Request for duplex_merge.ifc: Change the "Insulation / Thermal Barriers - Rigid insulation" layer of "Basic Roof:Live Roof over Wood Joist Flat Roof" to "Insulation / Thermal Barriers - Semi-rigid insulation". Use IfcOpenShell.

First a look at what the model holds.

```python
import ifcopenshell
import ifcopenshell.util.element

model = ifcopenshell.open("duplex_merge.ifc")
print(model.schema)
for layer_set in model.by_type("IfcMaterialLayerSet"):
    if layer_set.LayerSetName == "Basic Roof:Live Roof over Wood Joist Flat Roof":
        for layer in layer_set.MaterialLayers:
            print(layer.id(), layer.Material and layer.Material.Name, layer.LayerThickness, sep=" | ")
        print(len(ifcopenshell.util.element.get_elements_by_material(model, layer_set)), "elements and types use it")
print(sorted(m.Name for m in model.by_type("IfcMaterial") if m.Name)[:60])
```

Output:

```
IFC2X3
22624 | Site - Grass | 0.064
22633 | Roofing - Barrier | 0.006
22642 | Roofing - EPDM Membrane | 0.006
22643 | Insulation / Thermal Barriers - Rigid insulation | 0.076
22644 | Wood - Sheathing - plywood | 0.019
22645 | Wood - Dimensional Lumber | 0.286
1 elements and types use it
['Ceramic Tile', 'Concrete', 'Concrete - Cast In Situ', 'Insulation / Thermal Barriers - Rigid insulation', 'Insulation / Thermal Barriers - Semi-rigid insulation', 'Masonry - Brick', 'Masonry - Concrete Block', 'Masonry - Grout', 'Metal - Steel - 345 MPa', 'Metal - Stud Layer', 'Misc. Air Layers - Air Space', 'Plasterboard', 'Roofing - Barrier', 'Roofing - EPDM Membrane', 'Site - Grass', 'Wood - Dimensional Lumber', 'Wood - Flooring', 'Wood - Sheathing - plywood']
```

```python
import ifcopenshell
import ifcopenshell.api.material

model = ifcopenshell.open("duplex_merge.ifc")

layer_set = next(s for s in model.by_type("IfcMaterialLayerSet") if s.LayerSetName == "Basic Roof:Live Roof over Wood Joist Flat Roof")
layer = next(l for l in layer_set.MaterialLayers if l.Material and l.Material.Name == "Insulation / Thermal Barriers - Rigid insulation")
material = next(m for m in model.by_type("IfcMaterial") if m.Name == "Insulation / Thermal Barriers - Semi-rigid insulation")

# Point this one layer at the other material; renaming the old one would change it everywhere.
ifcopenshell.api.material.edit_layer(model, layer=layer, attributes={}, material=material)

print([l.Material.Name if l.Material else None for l in layer_set.MaterialLayers])

model.write("duplex_merge_edited.ifc")
```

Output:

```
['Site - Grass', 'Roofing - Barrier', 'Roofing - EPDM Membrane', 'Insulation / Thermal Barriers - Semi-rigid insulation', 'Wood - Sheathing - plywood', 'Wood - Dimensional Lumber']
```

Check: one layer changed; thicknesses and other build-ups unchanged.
